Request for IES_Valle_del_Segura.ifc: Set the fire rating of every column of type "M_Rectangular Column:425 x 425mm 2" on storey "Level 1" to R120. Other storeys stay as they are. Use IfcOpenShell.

First a look at what the model holds.

```python
import ifcopenshell
import ifcopenshell.util.element

model = ifcopenshell.open("IES_Valle_del_Segura.ifc")
print(model.schema)
storey = next(s for s in model.by_type("IfcBuildingStorey") if s.Name == "Level 1")
columns = [e for e in ifcopenshell.util.element.get_decomposition(storey) if e.is_a("IfcColumn")]
seen = {}
for e in columns:
    element_type = ifcopenshell.util.element.get_type(e)
    key = (element_type.Name if element_type != e and element_type else None, ifcopenshell.util.element.get_pset(e, "Pset_ColumnCommon", "FireRating"))
    seen[key] = seen.get(key, 0) + 1
for (name, value), count in sorted(seen.items(), key=str):
    print(count, "x", name, "|", value)
```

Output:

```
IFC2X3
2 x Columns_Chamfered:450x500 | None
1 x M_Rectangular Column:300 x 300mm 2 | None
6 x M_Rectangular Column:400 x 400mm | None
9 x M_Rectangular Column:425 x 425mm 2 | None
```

```python
import ifcopenshell
import ifcopenshell.api.pset
import ifcopenshell.util.element

model = ifcopenshell.open("IES_Valle_del_Segura.ifc")

storey = next(s for s in model.by_type("IfcBuildingStorey") if s.Name == "Level 1")
columns = [e for e in ifcopenshell.util.element.get_decomposition(storey) if e.is_a("IfcColumn")]

count = 0
for e in columns:
    element_type = ifcopenshell.util.element.get_type(e)
    if element_type in (None, e) or element_type.Name != "M_Rectangular Column:425 x 425mm 2":
        continue
    # add_pset returns the element's existing set when there is one.
    pset = ifcopenshell.api.pset.add_pset(model, product=e, name="Pset_ColumnCommon")
    ifcopenshell.api.pset.edit_pset(model, pset=pset, properties={"FireRating": "R120"})
    count += 1

print(count, "columns updated")

model.write("IES_Valle_del_Segura_edited.ifc")
```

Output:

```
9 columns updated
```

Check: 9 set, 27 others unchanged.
